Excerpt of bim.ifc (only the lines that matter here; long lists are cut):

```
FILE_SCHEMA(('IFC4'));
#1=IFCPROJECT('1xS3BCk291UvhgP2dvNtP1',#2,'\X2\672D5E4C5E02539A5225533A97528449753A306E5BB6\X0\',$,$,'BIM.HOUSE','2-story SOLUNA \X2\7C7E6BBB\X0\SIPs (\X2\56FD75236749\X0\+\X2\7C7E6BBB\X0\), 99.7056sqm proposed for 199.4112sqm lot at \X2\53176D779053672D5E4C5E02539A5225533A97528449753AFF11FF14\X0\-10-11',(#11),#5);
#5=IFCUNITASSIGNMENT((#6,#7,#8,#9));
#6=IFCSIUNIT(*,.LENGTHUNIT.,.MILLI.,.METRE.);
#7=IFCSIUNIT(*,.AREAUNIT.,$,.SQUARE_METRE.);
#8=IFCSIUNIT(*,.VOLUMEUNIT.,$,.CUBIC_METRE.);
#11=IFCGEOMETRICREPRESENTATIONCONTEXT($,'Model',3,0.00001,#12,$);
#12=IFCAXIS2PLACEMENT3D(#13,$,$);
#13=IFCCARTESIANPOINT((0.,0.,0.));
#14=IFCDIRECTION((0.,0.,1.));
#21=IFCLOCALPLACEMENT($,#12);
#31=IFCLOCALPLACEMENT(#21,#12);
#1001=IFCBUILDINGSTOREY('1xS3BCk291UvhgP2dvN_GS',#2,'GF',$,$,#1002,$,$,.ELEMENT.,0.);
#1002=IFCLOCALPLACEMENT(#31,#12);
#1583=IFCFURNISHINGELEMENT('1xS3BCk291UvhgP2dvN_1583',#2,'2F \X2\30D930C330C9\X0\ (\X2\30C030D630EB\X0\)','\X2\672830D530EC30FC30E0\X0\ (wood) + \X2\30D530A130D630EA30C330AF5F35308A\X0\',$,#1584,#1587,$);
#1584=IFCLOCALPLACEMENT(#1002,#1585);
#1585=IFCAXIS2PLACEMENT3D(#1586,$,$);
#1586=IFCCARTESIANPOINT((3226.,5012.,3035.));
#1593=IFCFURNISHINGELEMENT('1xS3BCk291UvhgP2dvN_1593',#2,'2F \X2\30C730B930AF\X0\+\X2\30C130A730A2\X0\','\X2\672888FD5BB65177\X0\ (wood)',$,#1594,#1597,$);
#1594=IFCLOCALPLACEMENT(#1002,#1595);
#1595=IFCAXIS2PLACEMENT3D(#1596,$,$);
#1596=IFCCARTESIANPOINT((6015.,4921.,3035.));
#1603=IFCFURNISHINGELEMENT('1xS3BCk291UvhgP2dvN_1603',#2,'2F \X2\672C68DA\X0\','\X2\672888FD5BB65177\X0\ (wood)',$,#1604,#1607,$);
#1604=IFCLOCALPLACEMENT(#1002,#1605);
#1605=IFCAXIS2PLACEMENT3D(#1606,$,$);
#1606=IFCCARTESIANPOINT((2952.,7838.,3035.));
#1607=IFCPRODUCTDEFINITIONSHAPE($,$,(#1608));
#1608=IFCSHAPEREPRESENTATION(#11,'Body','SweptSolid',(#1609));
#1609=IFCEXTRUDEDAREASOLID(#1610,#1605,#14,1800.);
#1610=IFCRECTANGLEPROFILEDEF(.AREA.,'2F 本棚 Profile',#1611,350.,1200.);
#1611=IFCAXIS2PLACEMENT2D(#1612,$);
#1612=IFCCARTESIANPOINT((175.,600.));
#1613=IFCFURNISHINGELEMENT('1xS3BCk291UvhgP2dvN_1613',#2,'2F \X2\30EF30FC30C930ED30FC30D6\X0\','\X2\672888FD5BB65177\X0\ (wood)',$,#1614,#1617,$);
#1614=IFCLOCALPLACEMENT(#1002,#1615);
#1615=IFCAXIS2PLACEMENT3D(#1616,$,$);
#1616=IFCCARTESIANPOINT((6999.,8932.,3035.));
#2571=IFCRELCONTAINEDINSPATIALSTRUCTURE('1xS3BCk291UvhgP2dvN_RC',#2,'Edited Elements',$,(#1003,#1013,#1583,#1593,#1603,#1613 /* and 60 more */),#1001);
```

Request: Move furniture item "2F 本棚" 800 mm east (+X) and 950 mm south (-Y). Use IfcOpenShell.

```python
import ifcopenshell
import ifcopenshell.api.geometry
import ifcopenshell.util.placement
import ifcopenshell.util.unit

model = ifcopenshell.open("bim.ifc")
unit_scale = ifcopenshell.util.unit.calculate_unit_scale(model)

item = model.by_id(1603)
matrix = ifcopenshell.util.placement.get_local_placement(item.ObjectPlacement)
matrix[0, 3] += 0.8 / unit_scale
matrix[1, 3] -= 0.95 / unit_scale
ifcopenshell.api.geometry.edit_object_placement(model, product=item, matrix=matrix, is_si=False)

print(ifcopenshell.util.placement.get_local_placement(item.ObjectPlacement).round(3) + 0.0)

model.write("bim-out.ifc")
```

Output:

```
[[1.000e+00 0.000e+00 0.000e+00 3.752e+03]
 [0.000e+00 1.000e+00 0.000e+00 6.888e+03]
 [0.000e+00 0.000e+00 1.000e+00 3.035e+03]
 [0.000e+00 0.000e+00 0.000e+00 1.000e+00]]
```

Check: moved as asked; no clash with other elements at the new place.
